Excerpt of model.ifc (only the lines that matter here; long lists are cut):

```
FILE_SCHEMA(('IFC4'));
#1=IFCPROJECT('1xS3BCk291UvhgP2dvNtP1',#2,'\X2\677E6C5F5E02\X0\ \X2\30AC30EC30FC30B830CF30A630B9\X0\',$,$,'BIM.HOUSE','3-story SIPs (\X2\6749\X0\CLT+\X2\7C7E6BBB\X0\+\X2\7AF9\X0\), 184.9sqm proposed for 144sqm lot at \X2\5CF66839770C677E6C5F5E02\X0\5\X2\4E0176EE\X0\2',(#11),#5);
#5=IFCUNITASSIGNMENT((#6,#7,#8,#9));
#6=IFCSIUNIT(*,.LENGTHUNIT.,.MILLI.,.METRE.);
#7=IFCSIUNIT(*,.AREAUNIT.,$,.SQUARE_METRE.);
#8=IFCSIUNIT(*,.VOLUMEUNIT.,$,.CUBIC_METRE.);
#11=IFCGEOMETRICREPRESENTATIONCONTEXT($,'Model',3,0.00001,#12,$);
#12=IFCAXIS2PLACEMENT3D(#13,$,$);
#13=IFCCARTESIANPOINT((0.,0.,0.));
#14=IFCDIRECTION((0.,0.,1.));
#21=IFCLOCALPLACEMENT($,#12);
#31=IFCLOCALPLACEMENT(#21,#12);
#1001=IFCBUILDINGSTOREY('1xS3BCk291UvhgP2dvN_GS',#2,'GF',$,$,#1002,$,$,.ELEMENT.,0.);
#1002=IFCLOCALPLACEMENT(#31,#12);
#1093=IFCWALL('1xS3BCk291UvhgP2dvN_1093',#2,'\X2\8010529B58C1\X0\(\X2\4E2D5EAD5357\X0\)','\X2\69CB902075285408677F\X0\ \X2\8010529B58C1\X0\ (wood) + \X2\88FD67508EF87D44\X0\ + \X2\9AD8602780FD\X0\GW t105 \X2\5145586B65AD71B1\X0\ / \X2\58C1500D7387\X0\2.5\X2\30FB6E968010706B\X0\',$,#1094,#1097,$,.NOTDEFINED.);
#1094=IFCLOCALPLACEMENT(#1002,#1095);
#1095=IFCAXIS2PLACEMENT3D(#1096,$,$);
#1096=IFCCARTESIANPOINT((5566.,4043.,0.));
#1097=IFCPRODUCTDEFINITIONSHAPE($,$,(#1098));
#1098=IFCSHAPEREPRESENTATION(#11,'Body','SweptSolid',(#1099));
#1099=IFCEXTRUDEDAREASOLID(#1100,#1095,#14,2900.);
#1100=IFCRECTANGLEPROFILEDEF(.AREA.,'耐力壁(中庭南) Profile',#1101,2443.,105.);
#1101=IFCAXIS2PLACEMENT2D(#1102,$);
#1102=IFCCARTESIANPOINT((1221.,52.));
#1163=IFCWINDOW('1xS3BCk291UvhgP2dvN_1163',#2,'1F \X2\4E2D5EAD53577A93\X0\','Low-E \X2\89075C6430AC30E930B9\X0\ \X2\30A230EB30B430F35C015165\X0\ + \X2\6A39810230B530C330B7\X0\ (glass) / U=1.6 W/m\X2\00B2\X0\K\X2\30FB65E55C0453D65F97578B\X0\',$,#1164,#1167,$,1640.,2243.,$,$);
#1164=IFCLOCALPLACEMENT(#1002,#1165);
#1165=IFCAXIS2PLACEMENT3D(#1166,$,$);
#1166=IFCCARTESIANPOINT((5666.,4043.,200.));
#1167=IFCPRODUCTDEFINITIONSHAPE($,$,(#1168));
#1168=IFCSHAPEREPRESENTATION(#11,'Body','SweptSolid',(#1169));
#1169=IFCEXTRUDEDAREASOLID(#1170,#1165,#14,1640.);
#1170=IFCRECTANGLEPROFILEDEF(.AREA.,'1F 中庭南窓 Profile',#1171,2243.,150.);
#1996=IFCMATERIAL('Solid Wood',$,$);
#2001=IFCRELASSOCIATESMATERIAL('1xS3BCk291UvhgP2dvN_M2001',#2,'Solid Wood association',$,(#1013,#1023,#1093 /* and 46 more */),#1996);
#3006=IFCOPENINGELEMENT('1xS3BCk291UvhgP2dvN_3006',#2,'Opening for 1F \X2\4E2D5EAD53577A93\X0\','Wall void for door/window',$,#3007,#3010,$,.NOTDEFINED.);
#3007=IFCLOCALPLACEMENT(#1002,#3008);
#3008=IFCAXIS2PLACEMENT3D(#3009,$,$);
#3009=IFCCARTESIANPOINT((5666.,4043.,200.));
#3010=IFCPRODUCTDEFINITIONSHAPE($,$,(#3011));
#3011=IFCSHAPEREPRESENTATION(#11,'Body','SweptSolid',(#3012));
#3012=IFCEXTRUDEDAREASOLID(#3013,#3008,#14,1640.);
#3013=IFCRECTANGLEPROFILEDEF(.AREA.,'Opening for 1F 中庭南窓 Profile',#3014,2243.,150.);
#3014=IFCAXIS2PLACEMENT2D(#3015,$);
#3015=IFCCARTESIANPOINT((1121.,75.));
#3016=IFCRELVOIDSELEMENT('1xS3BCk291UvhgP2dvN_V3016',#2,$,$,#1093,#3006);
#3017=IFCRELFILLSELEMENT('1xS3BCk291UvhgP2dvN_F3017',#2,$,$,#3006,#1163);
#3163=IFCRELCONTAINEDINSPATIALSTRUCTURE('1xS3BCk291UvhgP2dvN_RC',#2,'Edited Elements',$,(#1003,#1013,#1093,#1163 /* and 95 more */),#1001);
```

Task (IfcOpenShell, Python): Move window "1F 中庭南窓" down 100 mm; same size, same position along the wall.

```python
import numpy as np
import ifcopenshell
import ifcopenshell.api.geometry
import ifcopenshell.util.placement
import ifcopenshell.util.unit

model = ifcopenshell.open("model.ifc")
unit_scale = ifcopenshell.util.unit.calculate_unit_scale(model)

window = model.by_id(1163)
opening = window.FillsVoids[0].RelatingOpeningElement
dz = -100.0

shift = np.array([0.0, 0.0, dz])
# The window is not placed relative to its opening, so move both.
for product in (opening, window):
    matrix = ifcopenshell.util.placement.get_local_placement(product.ObjectPlacement)
    matrix[:3, 3] += shift
    ifcopenshell.api.geometry.edit_object_placement(model, product=product, matrix=matrix, is_si=False)

print(f"moved by {dz * unit_scale:+.3f} m")

model.write("model-out.ifc")
```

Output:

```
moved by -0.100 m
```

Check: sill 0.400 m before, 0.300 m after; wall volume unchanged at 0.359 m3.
